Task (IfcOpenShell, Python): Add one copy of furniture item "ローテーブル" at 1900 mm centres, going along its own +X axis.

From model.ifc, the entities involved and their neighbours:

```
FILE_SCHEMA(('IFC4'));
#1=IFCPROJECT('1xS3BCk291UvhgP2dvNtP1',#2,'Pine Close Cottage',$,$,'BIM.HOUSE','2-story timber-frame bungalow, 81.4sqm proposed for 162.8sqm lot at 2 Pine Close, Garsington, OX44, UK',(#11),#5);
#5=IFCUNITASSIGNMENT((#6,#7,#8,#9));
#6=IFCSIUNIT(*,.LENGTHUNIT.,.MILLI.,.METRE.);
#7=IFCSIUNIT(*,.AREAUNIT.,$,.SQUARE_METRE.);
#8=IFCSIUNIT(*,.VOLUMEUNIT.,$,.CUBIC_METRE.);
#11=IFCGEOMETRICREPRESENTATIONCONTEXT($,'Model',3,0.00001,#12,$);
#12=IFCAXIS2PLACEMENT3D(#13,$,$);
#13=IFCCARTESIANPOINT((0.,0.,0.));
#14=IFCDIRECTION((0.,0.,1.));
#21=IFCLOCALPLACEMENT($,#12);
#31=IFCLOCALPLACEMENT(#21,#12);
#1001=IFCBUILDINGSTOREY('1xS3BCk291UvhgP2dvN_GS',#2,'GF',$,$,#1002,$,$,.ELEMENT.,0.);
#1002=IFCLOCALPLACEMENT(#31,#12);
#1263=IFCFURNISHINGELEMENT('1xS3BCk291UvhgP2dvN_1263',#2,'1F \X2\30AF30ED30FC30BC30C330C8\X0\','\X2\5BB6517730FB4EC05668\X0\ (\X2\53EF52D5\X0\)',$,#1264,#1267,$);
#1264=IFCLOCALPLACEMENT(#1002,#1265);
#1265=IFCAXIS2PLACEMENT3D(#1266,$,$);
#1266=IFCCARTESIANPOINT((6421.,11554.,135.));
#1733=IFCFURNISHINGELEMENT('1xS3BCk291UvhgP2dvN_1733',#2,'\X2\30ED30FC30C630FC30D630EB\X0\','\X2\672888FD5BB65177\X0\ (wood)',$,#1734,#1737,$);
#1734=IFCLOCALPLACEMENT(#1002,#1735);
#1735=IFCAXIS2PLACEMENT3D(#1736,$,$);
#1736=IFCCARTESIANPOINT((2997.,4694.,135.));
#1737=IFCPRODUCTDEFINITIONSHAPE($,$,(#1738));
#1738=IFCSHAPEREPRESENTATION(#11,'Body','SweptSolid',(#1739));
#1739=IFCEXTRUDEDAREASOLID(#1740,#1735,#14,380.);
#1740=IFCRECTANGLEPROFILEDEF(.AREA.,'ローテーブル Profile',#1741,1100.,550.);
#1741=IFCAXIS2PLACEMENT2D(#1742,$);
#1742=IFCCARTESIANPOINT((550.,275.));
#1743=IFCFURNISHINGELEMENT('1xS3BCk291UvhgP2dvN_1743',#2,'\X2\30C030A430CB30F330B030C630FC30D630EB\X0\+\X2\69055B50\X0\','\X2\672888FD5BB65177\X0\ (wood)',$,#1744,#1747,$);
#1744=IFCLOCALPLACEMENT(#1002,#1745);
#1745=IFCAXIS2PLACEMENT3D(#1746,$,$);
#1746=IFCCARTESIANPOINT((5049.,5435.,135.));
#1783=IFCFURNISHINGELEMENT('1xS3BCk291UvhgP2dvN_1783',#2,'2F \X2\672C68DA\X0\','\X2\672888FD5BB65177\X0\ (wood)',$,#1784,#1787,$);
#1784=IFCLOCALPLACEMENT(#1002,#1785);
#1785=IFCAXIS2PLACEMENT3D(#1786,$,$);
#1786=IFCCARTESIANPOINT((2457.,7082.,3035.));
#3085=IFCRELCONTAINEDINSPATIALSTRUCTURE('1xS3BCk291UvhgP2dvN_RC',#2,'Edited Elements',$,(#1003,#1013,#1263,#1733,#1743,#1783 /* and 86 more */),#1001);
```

```python
import ifcopenshell
import ifcopenshell.api.geometry
import ifcopenshell.api.root
import ifcopenshell.util.element
import ifcopenshell.util.placement

model = ifcopenshell.open("model.ifc")


def reuse_history(source, copy):
    """copy_class also copies each property set's owner history, people and application; keep the originals."""
    for rel in copy.IsDefinedBy:
        if rel.is_a("IfcRelDefinesByProperties") and (history := rel.RelatingPropertyDefinition.OwnerHistory):
            rel.RelatingPropertyDefinition.OwnerHistory = source.OwnerHistory
            ifcopenshell.util.element.remove_deep2(model, history)


source = model.by_guid("1xS3BCk291UvhgP2dvN_1733")
base = ifcopenshell.util.placement.get_local_placement(source.ObjectPlacement)
step = base[:3, 0] * 1900.0

for i in range(1, 2):
    copy = ifcopenshell.api.root.copy_class(model, product=source)
    copy.Representation = ifcopenshell.util.element.copy_deep(
        model, source.Representation, exclude=["IfcGeometricRepresentationContext", "IfcRepresentationMap"]
    )
    reuse_history(source, copy)
    matrix = base.copy()
    matrix[:3, 3] += i * step
    print("added at", matrix[:3, 3].round(3) + 0.0)
    ifcopenshell.api.geometry.edit_object_placement(model, product=copy, matrix=matrix, is_si=False)

model.write("model_edited.ifc")
```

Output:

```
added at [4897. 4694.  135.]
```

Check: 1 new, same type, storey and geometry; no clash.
